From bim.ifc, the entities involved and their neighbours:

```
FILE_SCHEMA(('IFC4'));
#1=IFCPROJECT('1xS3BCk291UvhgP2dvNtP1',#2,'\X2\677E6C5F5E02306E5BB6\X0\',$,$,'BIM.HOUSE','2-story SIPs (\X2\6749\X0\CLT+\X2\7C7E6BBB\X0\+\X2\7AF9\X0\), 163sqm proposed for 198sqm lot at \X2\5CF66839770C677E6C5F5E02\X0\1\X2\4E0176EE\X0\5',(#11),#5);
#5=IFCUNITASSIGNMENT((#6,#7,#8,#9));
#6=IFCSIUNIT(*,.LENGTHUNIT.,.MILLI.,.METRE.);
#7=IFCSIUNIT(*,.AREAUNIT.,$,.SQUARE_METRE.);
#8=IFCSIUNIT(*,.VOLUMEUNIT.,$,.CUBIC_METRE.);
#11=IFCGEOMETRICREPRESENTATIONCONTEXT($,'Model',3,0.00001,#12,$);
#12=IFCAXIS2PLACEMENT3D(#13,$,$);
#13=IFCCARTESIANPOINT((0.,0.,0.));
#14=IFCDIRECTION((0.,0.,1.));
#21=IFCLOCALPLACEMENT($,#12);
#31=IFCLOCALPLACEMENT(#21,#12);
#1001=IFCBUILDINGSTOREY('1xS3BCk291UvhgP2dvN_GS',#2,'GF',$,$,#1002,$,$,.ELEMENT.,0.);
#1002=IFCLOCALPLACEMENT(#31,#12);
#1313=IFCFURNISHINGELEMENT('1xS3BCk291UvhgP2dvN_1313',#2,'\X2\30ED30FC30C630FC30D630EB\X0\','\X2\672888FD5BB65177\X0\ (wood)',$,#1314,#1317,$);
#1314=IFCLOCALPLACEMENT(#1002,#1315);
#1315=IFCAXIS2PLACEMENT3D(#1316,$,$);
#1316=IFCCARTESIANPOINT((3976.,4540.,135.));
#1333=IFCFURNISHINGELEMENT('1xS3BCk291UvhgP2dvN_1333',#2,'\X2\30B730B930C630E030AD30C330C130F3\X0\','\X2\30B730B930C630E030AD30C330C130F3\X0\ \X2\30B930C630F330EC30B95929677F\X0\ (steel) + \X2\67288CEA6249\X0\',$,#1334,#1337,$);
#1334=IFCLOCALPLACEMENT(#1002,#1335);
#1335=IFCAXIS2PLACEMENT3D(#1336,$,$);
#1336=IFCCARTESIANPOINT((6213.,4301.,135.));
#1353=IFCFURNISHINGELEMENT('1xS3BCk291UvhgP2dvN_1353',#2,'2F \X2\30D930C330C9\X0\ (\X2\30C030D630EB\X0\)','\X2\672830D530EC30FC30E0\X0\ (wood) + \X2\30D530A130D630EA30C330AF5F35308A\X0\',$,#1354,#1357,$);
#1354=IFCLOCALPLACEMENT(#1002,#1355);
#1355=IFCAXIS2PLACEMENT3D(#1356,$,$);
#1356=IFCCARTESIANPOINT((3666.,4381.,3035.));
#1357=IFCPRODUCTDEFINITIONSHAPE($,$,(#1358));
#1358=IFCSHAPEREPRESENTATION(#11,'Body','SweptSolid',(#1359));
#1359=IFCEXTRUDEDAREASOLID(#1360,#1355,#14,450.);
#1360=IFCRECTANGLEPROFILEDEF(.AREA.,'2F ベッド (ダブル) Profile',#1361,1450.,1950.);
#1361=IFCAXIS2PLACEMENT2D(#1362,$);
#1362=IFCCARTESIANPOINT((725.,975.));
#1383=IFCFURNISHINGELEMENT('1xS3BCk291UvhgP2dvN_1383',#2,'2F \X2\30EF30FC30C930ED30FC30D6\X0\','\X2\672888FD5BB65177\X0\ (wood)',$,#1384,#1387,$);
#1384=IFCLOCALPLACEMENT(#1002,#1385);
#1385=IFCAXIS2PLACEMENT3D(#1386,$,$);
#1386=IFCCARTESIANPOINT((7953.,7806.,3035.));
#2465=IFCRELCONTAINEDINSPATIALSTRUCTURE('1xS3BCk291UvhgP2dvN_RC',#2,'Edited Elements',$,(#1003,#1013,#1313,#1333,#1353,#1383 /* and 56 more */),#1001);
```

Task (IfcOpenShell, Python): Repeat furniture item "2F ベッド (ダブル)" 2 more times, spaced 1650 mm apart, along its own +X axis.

```python
import ifcopenshell
import ifcopenshell.api.geometry
import ifcopenshell.api.root
import ifcopenshell.util.element
import ifcopenshell.util.placement
import ifcopenshell.util.unit

model = ifcopenshell.open("bim.ifc")
unit_scale = ifcopenshell.util.unit.calculate_unit_scale(model)


def reuse_history(source, copy):
    """copy_class also copies each property set's owner history, people and application; keep the originals."""
    for rel in copy.IsDefinedBy:
        if rel.is_a("IfcRelDefinesByProperties") and (history := rel.RelatingPropertyDefinition.OwnerHistory):
            rel.RelatingPropertyDefinition.OwnerHistory = source.OwnerHistory
            ifcopenshell.util.element.remove_deep2(model, history)


source = model.by_id(1353)
base = ifcopenshell.util.placement.get_local_placement(source.ObjectPlacement)
step = base[:3, 0] * 1.65 / unit_scale

for i in range(1, 3):
    copy = ifcopenshell.api.root.copy_class(model, product=source)
    copy.Representation = ifcopenshell.util.element.copy_deep(
        model, source.Representation, exclude=["IfcGeometricRepresentationContext", "IfcRepresentationMap"]
    )
    reuse_history(source, copy)
    matrix = base.copy()
    matrix[:3, 3] += i * step
    print("added at", matrix[:3, 3].round(3) + 0.0)
    ifcopenshell.api.geometry.edit_object_placement(model, product=copy, matrix=matrix, is_si=False)

model.write("bim-out.ifc")
```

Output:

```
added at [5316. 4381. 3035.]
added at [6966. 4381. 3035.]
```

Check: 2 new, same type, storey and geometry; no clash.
